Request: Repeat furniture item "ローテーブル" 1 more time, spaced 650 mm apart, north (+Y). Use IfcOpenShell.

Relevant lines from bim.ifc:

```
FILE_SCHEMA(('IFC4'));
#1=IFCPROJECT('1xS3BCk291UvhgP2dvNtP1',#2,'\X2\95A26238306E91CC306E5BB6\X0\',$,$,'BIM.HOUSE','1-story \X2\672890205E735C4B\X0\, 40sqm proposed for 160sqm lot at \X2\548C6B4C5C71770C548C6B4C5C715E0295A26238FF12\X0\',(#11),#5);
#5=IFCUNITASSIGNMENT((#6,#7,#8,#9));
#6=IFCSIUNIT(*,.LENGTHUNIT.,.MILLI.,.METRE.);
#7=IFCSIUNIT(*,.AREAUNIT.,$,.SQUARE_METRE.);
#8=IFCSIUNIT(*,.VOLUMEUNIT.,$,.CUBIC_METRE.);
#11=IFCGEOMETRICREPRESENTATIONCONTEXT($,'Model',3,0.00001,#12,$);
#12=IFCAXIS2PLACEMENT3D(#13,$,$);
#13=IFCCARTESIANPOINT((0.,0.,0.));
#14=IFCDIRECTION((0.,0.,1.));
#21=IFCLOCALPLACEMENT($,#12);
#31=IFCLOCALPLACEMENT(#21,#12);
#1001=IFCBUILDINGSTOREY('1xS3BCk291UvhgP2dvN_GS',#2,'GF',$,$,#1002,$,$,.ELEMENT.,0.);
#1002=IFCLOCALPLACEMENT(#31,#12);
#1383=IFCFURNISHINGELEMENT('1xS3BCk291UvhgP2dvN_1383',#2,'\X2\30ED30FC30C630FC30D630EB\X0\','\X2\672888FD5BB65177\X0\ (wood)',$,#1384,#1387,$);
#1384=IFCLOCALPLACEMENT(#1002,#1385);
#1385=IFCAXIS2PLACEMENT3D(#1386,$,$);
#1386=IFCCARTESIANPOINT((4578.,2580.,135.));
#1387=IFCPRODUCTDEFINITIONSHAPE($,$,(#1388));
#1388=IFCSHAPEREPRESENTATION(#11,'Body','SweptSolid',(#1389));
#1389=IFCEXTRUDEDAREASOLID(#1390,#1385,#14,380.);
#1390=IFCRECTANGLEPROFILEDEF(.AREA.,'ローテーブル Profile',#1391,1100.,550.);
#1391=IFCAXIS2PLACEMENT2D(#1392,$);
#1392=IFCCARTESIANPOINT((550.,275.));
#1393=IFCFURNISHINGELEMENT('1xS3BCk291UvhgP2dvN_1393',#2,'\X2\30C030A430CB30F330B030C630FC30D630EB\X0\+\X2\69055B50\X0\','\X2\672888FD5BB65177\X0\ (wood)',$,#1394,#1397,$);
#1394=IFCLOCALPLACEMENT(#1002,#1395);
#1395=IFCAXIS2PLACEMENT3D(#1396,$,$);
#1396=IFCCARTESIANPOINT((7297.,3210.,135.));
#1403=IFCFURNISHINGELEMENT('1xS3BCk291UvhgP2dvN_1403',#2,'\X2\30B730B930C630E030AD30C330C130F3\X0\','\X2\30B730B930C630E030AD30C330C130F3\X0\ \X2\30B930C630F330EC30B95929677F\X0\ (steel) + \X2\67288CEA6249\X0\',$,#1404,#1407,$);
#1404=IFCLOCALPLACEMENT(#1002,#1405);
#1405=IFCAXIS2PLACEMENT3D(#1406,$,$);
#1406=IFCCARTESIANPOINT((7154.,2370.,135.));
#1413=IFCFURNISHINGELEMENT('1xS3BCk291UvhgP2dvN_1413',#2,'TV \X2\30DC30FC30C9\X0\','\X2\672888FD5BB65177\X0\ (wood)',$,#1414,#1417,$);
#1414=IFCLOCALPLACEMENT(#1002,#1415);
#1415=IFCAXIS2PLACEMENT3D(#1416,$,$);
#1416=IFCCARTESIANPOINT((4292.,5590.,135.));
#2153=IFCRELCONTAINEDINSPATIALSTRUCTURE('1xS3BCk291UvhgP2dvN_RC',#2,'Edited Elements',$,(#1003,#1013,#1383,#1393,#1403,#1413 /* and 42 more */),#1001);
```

```python
import numpy as np
import ifcopenshell
import ifcopenshell.api.geometry
import ifcopenshell.api.root
import ifcopenshell.util.element
import ifcopenshell.util.placement
import ifcopenshell.util.unit

model = ifcopenshell.open("bim.ifc")
unit_scale = ifcopenshell.util.unit.calculate_unit_scale(model)


def reuse_history(source, copy):
    """copy_class also copies each property set's owner history, people and application; keep the originals."""
    for rel in copy.IsDefinedBy:
        if rel.is_a("IfcRelDefinesByProperties") and (history := rel.RelatingPropertyDefinition.OwnerHistory):
            rel.RelatingPropertyDefinition.OwnerHistory = source.OwnerHistory
            ifcopenshell.util.element.remove_deep2(model, history)


source = model.by_guid("1xS3BCk291UvhgP2dvN_1383")
base = ifcopenshell.util.placement.get_local_placement(source.ObjectPlacement)
step = np.array([0.0, 1.0, 0.0]) * 0.65 / unit_scale

for i in range(1, 2):
    copy = ifcopenshell.api.root.copy_class(model, product=source)
    copy.Representation = ifcopenshell.util.element.copy_deep(
        model, source.Representation, exclude=["IfcGeometricRepresentationContext", "IfcRepresentationMap"]
    )
    reuse_history(source, copy)
    matrix = base.copy()
    matrix[:3, 3] += i * step
    print("added at", matrix[:3, 3].round(3) + 0.0)
    ifcopenshell.api.geometry.edit_object_placement(model, product=copy, matrix=matrix, is_si=False)

model.write("bim_updated.ifc")
```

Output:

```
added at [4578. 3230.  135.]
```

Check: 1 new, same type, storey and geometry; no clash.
